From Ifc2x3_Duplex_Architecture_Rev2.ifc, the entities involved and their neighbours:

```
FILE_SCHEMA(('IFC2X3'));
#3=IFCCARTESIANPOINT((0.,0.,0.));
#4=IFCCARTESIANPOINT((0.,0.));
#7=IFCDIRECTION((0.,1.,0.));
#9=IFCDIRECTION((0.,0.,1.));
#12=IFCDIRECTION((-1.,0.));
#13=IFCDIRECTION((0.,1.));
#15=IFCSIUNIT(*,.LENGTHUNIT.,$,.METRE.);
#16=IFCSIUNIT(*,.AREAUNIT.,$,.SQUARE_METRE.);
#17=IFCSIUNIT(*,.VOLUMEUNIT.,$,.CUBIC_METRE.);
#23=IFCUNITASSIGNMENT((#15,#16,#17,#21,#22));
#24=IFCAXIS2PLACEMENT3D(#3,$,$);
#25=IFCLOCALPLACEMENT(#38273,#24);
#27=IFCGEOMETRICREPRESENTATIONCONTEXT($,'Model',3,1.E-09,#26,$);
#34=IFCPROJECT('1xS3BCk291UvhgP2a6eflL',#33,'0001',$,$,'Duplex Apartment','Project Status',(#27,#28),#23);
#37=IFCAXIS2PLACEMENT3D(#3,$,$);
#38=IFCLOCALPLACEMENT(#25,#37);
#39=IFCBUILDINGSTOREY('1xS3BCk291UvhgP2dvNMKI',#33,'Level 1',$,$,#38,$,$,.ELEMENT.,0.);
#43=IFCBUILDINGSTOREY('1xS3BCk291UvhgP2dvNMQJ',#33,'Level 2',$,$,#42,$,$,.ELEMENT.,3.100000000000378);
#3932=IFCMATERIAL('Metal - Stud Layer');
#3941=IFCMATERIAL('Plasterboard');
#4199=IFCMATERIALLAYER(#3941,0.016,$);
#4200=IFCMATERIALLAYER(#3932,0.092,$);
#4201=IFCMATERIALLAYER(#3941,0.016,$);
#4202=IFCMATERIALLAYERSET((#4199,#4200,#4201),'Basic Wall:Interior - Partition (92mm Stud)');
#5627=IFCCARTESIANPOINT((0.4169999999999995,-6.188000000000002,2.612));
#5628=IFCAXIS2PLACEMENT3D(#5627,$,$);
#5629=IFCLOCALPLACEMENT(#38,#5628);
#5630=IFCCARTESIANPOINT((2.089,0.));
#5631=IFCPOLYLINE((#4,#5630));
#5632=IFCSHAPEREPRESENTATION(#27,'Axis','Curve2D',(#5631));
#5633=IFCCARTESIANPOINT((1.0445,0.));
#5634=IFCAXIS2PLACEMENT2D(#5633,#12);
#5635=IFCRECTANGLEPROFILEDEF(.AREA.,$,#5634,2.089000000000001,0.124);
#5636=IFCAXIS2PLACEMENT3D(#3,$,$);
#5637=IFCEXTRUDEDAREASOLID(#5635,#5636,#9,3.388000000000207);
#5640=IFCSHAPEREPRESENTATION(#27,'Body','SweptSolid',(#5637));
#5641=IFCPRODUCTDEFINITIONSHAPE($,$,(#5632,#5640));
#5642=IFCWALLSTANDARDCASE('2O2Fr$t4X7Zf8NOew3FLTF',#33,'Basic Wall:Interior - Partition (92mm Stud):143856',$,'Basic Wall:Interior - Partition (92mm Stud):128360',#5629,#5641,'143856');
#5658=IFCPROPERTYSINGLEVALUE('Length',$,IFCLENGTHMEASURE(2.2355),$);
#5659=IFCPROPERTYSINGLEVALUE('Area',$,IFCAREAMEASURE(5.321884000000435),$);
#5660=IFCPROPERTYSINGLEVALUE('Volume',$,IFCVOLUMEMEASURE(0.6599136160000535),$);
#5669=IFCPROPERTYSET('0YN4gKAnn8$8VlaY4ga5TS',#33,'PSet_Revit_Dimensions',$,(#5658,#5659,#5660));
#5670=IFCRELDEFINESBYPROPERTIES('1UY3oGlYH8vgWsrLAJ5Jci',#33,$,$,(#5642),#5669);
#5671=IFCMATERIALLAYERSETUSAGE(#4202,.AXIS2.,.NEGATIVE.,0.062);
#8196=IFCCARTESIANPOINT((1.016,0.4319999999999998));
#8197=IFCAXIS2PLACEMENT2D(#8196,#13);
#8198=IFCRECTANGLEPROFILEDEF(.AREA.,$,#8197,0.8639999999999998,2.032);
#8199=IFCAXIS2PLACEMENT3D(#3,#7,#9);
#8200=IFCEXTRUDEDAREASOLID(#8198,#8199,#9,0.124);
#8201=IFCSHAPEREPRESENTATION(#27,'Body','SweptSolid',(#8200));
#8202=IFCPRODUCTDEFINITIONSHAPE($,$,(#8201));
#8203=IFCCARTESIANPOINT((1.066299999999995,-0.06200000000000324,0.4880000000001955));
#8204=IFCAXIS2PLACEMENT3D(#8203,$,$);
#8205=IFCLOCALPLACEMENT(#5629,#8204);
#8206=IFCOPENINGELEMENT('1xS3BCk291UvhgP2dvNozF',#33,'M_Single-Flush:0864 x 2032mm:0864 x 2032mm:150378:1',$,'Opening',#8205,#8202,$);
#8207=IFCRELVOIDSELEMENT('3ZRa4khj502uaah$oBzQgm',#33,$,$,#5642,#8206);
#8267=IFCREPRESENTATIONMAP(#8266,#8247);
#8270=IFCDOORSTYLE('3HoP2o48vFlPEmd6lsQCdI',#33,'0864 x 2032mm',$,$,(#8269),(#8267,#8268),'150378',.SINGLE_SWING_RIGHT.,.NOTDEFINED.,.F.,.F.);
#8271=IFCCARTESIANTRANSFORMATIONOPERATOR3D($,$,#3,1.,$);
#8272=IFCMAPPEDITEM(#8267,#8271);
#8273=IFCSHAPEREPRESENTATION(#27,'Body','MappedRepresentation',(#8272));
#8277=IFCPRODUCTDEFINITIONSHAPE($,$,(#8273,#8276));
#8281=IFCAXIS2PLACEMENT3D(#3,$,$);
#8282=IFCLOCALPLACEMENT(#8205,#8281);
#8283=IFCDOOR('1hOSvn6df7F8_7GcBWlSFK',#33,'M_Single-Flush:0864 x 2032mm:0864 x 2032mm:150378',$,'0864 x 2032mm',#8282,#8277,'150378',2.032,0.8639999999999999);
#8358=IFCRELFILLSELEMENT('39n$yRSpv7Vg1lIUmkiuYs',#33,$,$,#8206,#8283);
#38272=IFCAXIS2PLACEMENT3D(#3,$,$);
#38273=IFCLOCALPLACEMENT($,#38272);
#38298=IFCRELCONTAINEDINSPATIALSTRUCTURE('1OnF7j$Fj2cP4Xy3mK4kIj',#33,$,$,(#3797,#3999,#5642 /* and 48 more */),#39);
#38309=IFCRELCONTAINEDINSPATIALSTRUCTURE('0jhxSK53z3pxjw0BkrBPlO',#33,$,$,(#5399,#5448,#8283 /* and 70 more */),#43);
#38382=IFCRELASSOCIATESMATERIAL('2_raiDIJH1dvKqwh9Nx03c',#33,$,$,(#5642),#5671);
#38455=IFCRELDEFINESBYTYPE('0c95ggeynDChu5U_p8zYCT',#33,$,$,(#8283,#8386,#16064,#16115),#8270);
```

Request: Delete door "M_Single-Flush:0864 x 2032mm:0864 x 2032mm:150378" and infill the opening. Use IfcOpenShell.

```python
import ifcopenshell
import ifcopenshell.api.feature
import ifcopenshell.api.pset
import ifcopenshell.api.root
import ifcopenshell.geom
import ifcopenshell.util.element
import ifcopenshell.util.shape
import ifcopenshell.util.unit

model = ifcopenshell.open("Ifc2x3_Duplex_Architecture_Rev2.ifc")
area_scale = ifcopenshell.util.unit.calculate_unit_scale(model, "AREAUNIT")
volume_scale = ifcopenshell.util.unit.calculate_unit_scale(model, "VOLUMEUNIT")
settings = ifcopenshell.geom.settings()


def volume(element):
    """Net volume in cubic metres, openings subtracted."""
    shape = ifcopenshell.geom.create_shape(settings, element)
    return ifcopenshell.util.shape.get_volume(shape.geometry)


door = model.by_id(8283)
opening = door.FillsVoids[0].RelatingOpeningElement
wall = opening.VoidsElements[0].RelatingBuildingElement
before = volume(wall)

ifcopenshell.api.root.remove_product(model, product=door)
ifcopenshell.api.feature.remove_feature(model, feature=opening)

after = volume(wall)
thickness = 0.124  # wall thickness in metres

# Update the wall's stored quantities.
pset = model.by_id(ifcopenshell.util.element.get_pset(wall, "PSet_Revit_Dimensions", should_inherit=False)["id"])
ifcopenshell.api.pset.edit_pset(model, pset=pset, properties={
    "Area": model.create_entity("IfcAreaMeasure", after / thickness / area_scale),
    "Volume": model.create_entity("IfcVolumeMeasure", after / volume_scale),
})

print(f"wall volume {before:.3f} -> {after:.3f} m3")

model.write("Ifc2x3_Duplex_Architecture_Rev2_v2.ifc")
```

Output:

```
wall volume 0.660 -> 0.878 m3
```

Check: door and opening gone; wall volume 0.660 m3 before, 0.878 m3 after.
